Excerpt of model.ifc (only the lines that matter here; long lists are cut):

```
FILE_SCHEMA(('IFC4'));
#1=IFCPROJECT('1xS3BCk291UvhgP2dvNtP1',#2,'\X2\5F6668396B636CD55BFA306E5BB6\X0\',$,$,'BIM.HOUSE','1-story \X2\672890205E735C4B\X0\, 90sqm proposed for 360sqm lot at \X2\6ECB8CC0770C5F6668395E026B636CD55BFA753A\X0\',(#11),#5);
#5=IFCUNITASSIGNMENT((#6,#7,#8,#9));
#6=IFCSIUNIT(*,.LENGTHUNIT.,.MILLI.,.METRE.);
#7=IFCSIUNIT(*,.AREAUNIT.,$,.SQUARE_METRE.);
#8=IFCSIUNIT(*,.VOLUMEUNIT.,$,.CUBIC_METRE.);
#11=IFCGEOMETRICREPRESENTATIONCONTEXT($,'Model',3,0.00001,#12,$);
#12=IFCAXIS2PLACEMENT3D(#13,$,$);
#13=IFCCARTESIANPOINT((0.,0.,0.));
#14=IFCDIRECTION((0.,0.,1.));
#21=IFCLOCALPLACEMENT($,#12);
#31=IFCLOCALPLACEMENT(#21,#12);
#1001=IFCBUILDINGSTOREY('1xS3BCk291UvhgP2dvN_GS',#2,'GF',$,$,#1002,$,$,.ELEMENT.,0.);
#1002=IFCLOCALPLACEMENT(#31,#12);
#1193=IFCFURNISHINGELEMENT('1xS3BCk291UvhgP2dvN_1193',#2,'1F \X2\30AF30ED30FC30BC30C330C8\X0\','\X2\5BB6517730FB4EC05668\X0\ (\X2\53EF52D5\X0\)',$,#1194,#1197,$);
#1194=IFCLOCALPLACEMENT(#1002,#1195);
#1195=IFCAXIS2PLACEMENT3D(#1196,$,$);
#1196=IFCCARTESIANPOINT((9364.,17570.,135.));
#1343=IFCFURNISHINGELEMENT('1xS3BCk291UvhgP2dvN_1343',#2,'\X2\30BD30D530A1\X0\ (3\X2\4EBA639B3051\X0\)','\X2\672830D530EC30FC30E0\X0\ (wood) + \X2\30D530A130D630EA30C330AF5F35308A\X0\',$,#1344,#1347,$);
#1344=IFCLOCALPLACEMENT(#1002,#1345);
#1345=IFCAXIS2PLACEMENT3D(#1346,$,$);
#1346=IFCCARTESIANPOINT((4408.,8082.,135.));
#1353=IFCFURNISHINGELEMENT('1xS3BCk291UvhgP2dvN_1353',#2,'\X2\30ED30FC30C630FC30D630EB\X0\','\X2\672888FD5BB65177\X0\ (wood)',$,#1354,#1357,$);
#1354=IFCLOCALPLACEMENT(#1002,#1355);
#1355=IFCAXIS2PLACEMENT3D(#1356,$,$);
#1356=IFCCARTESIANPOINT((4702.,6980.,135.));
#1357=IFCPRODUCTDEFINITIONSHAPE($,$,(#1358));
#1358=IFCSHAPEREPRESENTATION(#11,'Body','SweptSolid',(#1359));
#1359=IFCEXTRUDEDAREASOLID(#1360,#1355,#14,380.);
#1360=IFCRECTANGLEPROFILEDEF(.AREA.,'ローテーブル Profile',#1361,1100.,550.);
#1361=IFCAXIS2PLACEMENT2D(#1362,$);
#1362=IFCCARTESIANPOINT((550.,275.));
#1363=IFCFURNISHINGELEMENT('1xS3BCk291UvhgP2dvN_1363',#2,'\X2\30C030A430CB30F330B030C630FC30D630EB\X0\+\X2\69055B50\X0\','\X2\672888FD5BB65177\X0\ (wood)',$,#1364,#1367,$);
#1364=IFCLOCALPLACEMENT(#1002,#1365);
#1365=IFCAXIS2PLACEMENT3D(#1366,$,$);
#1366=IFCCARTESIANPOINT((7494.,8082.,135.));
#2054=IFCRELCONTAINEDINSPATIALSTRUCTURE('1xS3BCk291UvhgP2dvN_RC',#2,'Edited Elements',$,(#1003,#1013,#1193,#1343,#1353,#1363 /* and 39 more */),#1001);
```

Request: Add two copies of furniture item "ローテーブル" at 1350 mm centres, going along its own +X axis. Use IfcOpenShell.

```python
import ifcopenshell
import ifcopenshell.api.geometry
import ifcopenshell.api.root
import ifcopenshell.util.element
import ifcopenshell.util.placement
import ifcopenshell.util.unit

model = ifcopenshell.open("model.ifc")
unit_scale = ifcopenshell.util.unit.calculate_unit_scale(model)


def reuse_history(source, copy):
    """copy_class also copies each property set's owner history, people and application; keep the originals."""
    for rel in copy.IsDefinedBy:
        if rel.is_a("IfcRelDefinesByProperties") and (history := rel.RelatingPropertyDefinition.OwnerHistory):
            rel.RelatingPropertyDefinition.OwnerHistory = source.OwnerHistory
            ifcopenshell.util.element.remove_deep2(model, history)


source = model.by_id(1353)
base = ifcopenshell.util.placement.get_local_placement(source.ObjectPlacement)
step = base[:3, 0] * 1.35 / unit_scale

for i in range(1, 3):
    copy = ifcopenshell.api.root.copy_class(model, product=source)
    copy.Representation = ifcopenshell.util.element.copy_deep(
        model, source.Representation, exclude=["IfcGeometricRepresentationContext", "IfcRepresentationMap"]
    )
    reuse_history(source, copy)
    matrix = base.copy()
    matrix[:3, 3] += i * step
    print("added at", matrix[:3, 3].round(3) + 0.0)
    ifcopenshell.api.geometry.edit_object_placement(model, product=copy, matrix=matrix, is_si=False)

model.write("model-out.ifc")
```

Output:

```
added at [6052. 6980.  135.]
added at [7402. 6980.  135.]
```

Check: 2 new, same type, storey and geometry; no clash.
